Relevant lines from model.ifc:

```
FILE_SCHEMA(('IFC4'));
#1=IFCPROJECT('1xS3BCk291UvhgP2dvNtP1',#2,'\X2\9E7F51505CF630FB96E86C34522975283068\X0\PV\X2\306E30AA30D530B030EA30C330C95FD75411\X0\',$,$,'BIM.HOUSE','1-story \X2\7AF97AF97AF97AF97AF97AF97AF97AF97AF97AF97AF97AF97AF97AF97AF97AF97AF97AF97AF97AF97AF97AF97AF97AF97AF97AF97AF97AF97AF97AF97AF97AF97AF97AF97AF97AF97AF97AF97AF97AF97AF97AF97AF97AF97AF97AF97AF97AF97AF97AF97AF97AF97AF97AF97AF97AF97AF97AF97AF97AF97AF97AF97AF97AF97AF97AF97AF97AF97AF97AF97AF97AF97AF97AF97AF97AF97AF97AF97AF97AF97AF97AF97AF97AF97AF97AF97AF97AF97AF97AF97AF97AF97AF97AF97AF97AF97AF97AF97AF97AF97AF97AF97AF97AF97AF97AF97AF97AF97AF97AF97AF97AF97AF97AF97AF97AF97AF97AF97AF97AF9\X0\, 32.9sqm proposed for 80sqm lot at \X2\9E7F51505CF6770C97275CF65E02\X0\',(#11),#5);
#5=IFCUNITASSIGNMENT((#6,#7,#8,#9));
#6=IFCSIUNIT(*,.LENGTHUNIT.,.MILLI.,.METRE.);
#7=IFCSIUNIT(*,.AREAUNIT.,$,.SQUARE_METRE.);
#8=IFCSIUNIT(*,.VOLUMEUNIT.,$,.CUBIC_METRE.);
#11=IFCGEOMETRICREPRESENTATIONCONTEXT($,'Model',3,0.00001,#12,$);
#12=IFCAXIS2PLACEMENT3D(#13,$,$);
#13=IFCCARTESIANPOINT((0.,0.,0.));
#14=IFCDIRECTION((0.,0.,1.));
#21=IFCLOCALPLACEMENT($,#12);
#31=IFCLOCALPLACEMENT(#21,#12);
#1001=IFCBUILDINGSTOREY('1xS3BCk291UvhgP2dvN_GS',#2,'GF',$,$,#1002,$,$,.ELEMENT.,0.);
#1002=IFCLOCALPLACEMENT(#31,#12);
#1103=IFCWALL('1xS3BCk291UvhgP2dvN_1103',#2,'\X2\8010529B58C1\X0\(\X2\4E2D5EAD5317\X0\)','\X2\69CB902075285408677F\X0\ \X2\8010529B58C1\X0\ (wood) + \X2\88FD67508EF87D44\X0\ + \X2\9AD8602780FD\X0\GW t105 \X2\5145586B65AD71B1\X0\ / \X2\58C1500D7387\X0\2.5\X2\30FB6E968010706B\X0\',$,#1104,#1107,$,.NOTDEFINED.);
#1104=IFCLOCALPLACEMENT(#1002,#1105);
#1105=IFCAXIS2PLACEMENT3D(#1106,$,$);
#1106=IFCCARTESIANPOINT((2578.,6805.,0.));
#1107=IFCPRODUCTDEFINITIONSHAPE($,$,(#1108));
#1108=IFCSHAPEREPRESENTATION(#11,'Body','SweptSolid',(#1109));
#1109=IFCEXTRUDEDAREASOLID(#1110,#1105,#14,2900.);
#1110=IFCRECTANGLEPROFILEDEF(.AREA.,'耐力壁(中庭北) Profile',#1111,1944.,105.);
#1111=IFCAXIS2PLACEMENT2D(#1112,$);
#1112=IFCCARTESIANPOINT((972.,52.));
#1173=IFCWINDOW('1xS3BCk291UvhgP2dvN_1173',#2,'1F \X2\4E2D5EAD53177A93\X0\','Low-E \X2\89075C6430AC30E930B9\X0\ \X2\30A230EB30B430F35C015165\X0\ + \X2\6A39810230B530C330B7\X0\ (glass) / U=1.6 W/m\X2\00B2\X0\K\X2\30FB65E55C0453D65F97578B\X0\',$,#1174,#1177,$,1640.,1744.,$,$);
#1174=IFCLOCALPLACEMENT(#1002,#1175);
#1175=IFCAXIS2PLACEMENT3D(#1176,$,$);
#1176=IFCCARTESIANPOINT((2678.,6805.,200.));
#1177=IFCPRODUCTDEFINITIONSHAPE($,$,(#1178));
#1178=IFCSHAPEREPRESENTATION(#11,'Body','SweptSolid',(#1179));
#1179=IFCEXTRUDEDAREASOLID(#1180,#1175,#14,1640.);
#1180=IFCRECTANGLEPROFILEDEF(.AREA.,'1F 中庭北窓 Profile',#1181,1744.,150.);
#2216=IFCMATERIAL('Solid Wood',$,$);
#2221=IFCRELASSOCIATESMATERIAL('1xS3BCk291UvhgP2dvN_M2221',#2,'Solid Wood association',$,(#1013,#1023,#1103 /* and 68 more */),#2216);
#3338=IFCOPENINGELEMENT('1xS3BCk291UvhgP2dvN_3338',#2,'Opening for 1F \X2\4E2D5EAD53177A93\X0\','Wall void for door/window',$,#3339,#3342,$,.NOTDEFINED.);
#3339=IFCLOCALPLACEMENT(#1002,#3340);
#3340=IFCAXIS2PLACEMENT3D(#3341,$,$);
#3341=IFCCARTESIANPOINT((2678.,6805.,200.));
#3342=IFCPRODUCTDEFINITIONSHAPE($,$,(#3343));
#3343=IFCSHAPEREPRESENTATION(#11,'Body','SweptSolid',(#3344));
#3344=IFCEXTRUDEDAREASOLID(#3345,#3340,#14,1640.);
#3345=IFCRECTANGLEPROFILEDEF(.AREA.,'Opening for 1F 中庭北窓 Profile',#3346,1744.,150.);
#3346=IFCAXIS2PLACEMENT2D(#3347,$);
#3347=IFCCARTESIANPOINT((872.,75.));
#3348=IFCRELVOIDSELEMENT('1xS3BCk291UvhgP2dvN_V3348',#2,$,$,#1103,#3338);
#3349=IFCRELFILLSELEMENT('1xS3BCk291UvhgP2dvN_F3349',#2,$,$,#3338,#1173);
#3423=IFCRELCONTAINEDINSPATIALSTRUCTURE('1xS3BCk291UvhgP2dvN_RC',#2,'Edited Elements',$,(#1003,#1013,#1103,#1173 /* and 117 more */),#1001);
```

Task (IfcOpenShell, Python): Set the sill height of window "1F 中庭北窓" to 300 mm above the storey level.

```python
import numpy as np
import ifcopenshell
import ifcopenshell.api.geometry
import ifcopenshell.geom
import ifcopenshell.util.element
import ifcopenshell.util.placement
import ifcopenshell.util.shape
import ifcopenshell.util.unit

model = ifcopenshell.open("model.ifc")
unit_scale = ifcopenshell.util.unit.calculate_unit_scale(model)

window = model.by_id(1173)
opening = window.FillsVoids[0].RelatingOpeningElement
storey = ifcopenshell.util.element.get_container(window, ifc_class="IfcBuildingStorey")
level = ifcopenshell.util.placement.get_local_placement(storey.ObjectPlacement)[2, 3]

# The opening's origin need not be at the sill, so measure its lowest point.
shape = ifcopenshell.geom.create_shape(ifcopenshell.geom.settings(), opening)
bottom = ifcopenshell.util.shape.get_shape_bottom_elevation(shape, shape.geometry) / unit_scale
dz = level + 300.0 - bottom

shift = np.array([0.0, 0.0, dz])
# The window is not placed relative to its opening, so move both.
for product in (opening, window):
    matrix = ifcopenshell.util.placement.get_local_placement(product.ObjectPlacement)
    matrix[:3, 3] += shift
    ifcopenshell.api.geometry.edit_object_placement(model, product=product, matrix=matrix, is_si=False)

print(f"moved by {dz * unit_scale:+.3f} m")

model.write("model-out.ifc")
```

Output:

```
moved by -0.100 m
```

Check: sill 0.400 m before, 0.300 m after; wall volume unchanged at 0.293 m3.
